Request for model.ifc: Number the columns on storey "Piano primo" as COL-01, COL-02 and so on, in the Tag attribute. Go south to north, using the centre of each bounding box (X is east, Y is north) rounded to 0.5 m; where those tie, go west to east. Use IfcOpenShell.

First a look at what the model holds.

```python
import ifcopenshell
import ifcopenshell.util.element
import ifcopenshell.util.placement

model = ifcopenshell.open("model.ifc")
print(model.schema)
storey = next(s for s in model.by_type("IfcBuildingStorey") if s.Name == "Piano primo")
columns = [e for e in ifcopenshell.util.element.get_decomposition(storey) if e.is_a("IfcColumn")]
for e in sorted(columns, key=lambda e: e.id()):
    origin = ifcopenshell.util.placement.get_local_placement(e.ObjectPlacement)[:3, 3]
    print(e.id(), e.Tag, e.Name, origin.round(2) + 0.0, sep=" | ")
```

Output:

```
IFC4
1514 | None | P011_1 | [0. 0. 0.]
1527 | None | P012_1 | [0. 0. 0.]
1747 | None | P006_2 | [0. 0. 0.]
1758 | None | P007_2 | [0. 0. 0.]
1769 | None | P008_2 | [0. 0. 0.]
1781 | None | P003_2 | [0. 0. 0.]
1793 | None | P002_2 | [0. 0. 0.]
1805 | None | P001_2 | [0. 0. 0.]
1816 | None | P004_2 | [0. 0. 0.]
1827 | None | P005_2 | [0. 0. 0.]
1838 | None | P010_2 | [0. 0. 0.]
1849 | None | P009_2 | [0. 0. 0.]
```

```python
import ifcopenshell
import ifcopenshell.geom
import ifcopenshell.util.element
import ifcopenshell.util.shape

model = ifcopenshell.open("model.ifc")
settings = ifcopenshell.geom.settings()
settings.set("use-world-coords", True)


def centre(element):
    shape = ifcopenshell.geom.create_shape(settings, element)
    return ifcopenshell.util.shape.get_bbox_centroid(shape.geometry)


storey = next(s for s in model.by_type("IfcBuildingStorey") if s.Name == "Piano primo")
columns = [e for e in ifcopenshell.util.element.get_decomposition(storey) if e.is_a("IfcColumn")]

# Insertion points can sit at a corner or the storey origin, so sort by the geometry (in metres).
centres = {e: centre(e) for e in columns}
columns.sort(key=lambda e: (round(centres[e][1] / 0.5), centres[e][0]))

for i, e in enumerate(columns, start=1):
    number = f"COL-{i:02d}"
    e.Tag = number
    print(e.id(), number)

model.write("model_v2.ifc")
```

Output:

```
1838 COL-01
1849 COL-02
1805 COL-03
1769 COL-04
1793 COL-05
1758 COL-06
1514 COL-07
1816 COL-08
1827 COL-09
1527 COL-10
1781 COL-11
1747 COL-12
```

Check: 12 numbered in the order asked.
